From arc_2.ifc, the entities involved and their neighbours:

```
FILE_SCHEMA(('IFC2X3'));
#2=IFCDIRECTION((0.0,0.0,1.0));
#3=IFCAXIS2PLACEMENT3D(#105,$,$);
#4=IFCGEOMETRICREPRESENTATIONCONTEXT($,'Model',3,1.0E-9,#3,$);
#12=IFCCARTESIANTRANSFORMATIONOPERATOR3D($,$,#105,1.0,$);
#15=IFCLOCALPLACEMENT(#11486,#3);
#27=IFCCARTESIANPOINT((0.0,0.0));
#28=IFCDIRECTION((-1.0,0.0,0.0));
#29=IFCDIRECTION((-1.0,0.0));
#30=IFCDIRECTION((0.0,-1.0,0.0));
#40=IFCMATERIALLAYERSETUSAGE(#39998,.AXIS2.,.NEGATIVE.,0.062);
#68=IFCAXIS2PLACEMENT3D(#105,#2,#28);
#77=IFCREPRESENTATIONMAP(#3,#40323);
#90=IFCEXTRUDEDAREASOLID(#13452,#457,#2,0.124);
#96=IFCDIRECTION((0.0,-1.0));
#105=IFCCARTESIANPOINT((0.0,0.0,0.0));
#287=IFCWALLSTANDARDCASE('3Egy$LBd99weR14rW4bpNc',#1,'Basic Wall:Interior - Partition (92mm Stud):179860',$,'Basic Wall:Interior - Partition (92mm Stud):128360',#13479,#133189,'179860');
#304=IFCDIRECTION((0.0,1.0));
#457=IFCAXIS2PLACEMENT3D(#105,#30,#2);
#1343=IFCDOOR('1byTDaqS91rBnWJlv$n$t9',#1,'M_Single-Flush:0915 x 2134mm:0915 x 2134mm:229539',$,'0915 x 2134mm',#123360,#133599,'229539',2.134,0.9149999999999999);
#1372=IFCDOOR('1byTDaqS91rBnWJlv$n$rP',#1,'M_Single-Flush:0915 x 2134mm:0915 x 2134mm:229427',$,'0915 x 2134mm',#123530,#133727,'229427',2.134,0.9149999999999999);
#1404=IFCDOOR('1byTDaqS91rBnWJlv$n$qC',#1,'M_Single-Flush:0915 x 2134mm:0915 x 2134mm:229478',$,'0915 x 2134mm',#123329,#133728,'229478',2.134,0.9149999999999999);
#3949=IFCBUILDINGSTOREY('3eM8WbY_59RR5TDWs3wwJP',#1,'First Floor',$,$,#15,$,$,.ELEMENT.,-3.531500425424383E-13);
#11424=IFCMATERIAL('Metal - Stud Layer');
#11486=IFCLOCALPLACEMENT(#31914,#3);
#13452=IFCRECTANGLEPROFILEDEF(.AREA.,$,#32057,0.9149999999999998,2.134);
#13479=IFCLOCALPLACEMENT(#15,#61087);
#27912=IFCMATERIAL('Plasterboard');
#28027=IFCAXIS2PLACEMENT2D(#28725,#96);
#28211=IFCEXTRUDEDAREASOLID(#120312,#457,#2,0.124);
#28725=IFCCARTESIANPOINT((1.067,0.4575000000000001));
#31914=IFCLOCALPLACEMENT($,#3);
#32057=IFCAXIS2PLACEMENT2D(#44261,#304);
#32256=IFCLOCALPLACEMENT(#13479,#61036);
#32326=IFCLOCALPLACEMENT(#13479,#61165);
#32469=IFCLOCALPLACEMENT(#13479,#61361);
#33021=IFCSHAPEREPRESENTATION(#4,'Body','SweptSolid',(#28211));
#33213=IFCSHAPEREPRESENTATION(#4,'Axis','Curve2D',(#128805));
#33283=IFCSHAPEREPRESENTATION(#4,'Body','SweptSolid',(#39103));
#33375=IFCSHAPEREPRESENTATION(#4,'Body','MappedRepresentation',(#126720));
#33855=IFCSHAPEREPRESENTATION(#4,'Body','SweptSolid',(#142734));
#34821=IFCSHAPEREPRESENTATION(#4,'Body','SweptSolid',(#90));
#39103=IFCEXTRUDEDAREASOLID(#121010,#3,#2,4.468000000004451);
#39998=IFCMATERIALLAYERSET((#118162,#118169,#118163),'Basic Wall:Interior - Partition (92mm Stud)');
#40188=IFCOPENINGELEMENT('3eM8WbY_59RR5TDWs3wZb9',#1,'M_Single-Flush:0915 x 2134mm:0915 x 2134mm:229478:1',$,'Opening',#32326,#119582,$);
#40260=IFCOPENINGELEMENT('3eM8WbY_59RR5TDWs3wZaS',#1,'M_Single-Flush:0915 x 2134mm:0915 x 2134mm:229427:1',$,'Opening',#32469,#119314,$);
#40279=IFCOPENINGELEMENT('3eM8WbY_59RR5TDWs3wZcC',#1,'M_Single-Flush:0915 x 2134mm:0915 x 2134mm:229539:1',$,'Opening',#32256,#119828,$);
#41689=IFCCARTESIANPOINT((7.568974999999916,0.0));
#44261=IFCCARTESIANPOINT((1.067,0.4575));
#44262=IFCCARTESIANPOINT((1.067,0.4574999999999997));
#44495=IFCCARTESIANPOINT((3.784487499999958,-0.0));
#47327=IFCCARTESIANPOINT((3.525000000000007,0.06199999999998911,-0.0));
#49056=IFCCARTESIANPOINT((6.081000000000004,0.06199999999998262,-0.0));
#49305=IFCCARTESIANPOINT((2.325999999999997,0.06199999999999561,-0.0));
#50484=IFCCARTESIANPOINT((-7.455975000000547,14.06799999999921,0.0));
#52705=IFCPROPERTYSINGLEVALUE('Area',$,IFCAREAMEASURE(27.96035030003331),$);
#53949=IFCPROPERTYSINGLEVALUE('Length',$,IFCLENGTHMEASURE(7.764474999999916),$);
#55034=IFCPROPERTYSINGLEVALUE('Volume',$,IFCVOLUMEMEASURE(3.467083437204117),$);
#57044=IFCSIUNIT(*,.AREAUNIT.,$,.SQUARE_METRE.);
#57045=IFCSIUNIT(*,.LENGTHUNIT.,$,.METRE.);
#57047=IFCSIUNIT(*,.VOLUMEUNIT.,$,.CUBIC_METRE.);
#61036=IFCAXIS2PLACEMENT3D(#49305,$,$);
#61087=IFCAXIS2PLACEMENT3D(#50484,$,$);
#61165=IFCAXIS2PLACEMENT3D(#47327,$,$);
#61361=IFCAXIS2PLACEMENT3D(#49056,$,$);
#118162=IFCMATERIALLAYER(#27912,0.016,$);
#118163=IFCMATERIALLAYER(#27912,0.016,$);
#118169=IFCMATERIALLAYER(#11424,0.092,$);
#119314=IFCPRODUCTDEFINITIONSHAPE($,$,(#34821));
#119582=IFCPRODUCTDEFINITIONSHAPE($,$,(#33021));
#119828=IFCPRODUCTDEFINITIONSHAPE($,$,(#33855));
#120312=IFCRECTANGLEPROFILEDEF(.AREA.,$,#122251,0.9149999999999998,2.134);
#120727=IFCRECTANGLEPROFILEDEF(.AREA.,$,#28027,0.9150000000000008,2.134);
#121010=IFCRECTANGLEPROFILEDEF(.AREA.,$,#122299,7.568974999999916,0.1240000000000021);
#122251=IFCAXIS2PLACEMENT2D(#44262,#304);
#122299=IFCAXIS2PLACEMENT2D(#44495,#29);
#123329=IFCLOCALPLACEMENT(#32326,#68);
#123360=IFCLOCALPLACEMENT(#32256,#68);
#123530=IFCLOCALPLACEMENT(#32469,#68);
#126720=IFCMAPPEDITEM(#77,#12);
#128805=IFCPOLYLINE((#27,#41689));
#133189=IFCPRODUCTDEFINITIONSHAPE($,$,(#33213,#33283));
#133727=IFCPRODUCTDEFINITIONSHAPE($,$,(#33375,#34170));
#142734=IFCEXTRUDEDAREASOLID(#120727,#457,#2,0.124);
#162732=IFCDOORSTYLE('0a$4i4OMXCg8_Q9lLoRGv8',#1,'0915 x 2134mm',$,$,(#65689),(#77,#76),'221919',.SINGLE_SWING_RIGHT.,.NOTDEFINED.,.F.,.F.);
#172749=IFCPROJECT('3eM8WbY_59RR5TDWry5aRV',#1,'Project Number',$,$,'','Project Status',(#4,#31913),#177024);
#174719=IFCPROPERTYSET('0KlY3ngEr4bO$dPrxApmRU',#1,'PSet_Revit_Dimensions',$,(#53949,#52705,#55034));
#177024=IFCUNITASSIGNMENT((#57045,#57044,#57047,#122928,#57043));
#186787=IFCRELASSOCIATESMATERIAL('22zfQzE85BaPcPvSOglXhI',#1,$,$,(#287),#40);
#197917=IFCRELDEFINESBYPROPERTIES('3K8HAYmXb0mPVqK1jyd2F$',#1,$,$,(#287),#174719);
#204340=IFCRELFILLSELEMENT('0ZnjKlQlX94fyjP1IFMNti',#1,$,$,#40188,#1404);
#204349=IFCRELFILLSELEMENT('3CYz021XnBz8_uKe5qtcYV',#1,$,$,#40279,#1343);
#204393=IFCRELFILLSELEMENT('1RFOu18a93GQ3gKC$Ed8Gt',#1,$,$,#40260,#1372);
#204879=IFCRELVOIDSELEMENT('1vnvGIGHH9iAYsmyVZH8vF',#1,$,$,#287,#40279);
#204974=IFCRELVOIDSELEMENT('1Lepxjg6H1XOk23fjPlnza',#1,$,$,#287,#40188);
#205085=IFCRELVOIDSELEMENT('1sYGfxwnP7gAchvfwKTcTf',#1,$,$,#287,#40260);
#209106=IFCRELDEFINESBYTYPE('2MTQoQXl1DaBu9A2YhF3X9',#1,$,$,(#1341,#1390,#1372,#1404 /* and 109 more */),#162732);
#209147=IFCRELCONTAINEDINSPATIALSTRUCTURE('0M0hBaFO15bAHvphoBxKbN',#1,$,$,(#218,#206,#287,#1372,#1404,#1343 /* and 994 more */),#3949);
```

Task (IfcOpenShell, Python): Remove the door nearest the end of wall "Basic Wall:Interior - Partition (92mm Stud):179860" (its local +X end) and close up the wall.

```python
import ifcopenshell
import ifcopenshell.api.feature
import ifcopenshell.api.pset
import ifcopenshell.api.root
import ifcopenshell.geom
import ifcopenshell.util.element
import ifcopenshell.util.shape
import ifcopenshell.util.unit

model = ifcopenshell.open("arc_2.ifc")
area_scale = ifcopenshell.util.unit.calculate_unit_scale(model, "AREAUNIT")
volume_scale = ifcopenshell.util.unit.calculate_unit_scale(model, "VOLUMEUNIT")
settings = ifcopenshell.geom.settings()


def volume(element):
    """Net volume in cubic metres, openings subtracted."""
    shape = ifcopenshell.geom.create_shape(settings, element)
    return ifcopenshell.util.shape.get_volume(shape.geometry)


door = model.by_id(1372)
opening = door.FillsVoids[0].RelatingOpeningElement
wall = opening.VoidsElements[0].RelatingBuildingElement
before = volume(wall)

ifcopenshell.api.root.remove_product(model, product=door)
ifcopenshell.api.feature.remove_feature(model, feature=opening)

after = volume(wall)
thickness = 0.124  # wall thickness in metres

# Update the wall's stored quantities.
pset = model.by_id(ifcopenshell.util.element.get_pset(wall, "PSet_Revit_Dimensions", should_inherit=False)["id"])
ifcopenshell.api.pset.edit_pset(model, pset=pset, properties={
    "Area": model.create_entity("IfcAreaMeasure", after / thickness / area_scale),
    "Volume": model.create_entity("IfcVolumeMeasure", after / volume_scale),
})

print(f"wall volume {before:.3f} -> {after:.3f} m3")

model.write("arc_2_rev.ifc")
```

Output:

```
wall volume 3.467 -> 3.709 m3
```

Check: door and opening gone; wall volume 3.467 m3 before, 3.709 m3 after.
